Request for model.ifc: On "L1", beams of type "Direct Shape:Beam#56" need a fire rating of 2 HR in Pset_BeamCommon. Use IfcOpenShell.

First a look at what the model holds.

```python
import ifcopenshell
import ifcopenshell.util.element

model = ifcopenshell.open("model.ifc")
print(model.schema)
storey = next(s for s in model.by_type("IfcBuildingStorey") if s.Name == "L1")
beams = [e for e in ifcopenshell.util.element.get_decomposition(storey) if e.is_a("IfcBeam")]
seen = {}
for e in beams:
    element_type = ifcopenshell.util.element.get_type(e)
    key = (element_type.Name if element_type != e and element_type else None, ifcopenshell.util.element.get_pset(e, "Pset_BeamCommon", "FireRating"))
    seen[key] = seen.get(key, 0) + 1
for (name, value), count in sorted(seen.items(), key=str):
    print(count, "x", name, "|", value)
```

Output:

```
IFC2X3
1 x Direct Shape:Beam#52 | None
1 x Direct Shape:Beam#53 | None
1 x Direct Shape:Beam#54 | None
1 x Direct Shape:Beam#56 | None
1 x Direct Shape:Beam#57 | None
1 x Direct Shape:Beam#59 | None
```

```python
import ifcopenshell
import ifcopenshell.api.pset
import ifcopenshell.util.element

model = ifcopenshell.open("model.ifc")

storey = next(s for s in model.by_type("IfcBuildingStorey") if s.Name == "L1")
beams = [e for e in ifcopenshell.util.element.get_decomposition(storey) if e.is_a("IfcBeam")]

count = 0
for e in beams:
    element_type = ifcopenshell.util.element.get_type(e)
    if element_type in (None, e) or element_type.Name != "Direct Shape:Beam#56":
        continue
    # add_pset returns the element's existing set when there is one.
    pset = ifcopenshell.api.pset.add_pset(model, product=e, name="Pset_BeamCommon")
    ifcopenshell.api.pset.edit_pset(model, pset=pset, properties={"FireRating": "2 HR"})
    count += 1

print(count, "beams updated")

model.write("model-out.ifc")
```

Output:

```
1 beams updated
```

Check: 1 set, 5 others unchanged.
